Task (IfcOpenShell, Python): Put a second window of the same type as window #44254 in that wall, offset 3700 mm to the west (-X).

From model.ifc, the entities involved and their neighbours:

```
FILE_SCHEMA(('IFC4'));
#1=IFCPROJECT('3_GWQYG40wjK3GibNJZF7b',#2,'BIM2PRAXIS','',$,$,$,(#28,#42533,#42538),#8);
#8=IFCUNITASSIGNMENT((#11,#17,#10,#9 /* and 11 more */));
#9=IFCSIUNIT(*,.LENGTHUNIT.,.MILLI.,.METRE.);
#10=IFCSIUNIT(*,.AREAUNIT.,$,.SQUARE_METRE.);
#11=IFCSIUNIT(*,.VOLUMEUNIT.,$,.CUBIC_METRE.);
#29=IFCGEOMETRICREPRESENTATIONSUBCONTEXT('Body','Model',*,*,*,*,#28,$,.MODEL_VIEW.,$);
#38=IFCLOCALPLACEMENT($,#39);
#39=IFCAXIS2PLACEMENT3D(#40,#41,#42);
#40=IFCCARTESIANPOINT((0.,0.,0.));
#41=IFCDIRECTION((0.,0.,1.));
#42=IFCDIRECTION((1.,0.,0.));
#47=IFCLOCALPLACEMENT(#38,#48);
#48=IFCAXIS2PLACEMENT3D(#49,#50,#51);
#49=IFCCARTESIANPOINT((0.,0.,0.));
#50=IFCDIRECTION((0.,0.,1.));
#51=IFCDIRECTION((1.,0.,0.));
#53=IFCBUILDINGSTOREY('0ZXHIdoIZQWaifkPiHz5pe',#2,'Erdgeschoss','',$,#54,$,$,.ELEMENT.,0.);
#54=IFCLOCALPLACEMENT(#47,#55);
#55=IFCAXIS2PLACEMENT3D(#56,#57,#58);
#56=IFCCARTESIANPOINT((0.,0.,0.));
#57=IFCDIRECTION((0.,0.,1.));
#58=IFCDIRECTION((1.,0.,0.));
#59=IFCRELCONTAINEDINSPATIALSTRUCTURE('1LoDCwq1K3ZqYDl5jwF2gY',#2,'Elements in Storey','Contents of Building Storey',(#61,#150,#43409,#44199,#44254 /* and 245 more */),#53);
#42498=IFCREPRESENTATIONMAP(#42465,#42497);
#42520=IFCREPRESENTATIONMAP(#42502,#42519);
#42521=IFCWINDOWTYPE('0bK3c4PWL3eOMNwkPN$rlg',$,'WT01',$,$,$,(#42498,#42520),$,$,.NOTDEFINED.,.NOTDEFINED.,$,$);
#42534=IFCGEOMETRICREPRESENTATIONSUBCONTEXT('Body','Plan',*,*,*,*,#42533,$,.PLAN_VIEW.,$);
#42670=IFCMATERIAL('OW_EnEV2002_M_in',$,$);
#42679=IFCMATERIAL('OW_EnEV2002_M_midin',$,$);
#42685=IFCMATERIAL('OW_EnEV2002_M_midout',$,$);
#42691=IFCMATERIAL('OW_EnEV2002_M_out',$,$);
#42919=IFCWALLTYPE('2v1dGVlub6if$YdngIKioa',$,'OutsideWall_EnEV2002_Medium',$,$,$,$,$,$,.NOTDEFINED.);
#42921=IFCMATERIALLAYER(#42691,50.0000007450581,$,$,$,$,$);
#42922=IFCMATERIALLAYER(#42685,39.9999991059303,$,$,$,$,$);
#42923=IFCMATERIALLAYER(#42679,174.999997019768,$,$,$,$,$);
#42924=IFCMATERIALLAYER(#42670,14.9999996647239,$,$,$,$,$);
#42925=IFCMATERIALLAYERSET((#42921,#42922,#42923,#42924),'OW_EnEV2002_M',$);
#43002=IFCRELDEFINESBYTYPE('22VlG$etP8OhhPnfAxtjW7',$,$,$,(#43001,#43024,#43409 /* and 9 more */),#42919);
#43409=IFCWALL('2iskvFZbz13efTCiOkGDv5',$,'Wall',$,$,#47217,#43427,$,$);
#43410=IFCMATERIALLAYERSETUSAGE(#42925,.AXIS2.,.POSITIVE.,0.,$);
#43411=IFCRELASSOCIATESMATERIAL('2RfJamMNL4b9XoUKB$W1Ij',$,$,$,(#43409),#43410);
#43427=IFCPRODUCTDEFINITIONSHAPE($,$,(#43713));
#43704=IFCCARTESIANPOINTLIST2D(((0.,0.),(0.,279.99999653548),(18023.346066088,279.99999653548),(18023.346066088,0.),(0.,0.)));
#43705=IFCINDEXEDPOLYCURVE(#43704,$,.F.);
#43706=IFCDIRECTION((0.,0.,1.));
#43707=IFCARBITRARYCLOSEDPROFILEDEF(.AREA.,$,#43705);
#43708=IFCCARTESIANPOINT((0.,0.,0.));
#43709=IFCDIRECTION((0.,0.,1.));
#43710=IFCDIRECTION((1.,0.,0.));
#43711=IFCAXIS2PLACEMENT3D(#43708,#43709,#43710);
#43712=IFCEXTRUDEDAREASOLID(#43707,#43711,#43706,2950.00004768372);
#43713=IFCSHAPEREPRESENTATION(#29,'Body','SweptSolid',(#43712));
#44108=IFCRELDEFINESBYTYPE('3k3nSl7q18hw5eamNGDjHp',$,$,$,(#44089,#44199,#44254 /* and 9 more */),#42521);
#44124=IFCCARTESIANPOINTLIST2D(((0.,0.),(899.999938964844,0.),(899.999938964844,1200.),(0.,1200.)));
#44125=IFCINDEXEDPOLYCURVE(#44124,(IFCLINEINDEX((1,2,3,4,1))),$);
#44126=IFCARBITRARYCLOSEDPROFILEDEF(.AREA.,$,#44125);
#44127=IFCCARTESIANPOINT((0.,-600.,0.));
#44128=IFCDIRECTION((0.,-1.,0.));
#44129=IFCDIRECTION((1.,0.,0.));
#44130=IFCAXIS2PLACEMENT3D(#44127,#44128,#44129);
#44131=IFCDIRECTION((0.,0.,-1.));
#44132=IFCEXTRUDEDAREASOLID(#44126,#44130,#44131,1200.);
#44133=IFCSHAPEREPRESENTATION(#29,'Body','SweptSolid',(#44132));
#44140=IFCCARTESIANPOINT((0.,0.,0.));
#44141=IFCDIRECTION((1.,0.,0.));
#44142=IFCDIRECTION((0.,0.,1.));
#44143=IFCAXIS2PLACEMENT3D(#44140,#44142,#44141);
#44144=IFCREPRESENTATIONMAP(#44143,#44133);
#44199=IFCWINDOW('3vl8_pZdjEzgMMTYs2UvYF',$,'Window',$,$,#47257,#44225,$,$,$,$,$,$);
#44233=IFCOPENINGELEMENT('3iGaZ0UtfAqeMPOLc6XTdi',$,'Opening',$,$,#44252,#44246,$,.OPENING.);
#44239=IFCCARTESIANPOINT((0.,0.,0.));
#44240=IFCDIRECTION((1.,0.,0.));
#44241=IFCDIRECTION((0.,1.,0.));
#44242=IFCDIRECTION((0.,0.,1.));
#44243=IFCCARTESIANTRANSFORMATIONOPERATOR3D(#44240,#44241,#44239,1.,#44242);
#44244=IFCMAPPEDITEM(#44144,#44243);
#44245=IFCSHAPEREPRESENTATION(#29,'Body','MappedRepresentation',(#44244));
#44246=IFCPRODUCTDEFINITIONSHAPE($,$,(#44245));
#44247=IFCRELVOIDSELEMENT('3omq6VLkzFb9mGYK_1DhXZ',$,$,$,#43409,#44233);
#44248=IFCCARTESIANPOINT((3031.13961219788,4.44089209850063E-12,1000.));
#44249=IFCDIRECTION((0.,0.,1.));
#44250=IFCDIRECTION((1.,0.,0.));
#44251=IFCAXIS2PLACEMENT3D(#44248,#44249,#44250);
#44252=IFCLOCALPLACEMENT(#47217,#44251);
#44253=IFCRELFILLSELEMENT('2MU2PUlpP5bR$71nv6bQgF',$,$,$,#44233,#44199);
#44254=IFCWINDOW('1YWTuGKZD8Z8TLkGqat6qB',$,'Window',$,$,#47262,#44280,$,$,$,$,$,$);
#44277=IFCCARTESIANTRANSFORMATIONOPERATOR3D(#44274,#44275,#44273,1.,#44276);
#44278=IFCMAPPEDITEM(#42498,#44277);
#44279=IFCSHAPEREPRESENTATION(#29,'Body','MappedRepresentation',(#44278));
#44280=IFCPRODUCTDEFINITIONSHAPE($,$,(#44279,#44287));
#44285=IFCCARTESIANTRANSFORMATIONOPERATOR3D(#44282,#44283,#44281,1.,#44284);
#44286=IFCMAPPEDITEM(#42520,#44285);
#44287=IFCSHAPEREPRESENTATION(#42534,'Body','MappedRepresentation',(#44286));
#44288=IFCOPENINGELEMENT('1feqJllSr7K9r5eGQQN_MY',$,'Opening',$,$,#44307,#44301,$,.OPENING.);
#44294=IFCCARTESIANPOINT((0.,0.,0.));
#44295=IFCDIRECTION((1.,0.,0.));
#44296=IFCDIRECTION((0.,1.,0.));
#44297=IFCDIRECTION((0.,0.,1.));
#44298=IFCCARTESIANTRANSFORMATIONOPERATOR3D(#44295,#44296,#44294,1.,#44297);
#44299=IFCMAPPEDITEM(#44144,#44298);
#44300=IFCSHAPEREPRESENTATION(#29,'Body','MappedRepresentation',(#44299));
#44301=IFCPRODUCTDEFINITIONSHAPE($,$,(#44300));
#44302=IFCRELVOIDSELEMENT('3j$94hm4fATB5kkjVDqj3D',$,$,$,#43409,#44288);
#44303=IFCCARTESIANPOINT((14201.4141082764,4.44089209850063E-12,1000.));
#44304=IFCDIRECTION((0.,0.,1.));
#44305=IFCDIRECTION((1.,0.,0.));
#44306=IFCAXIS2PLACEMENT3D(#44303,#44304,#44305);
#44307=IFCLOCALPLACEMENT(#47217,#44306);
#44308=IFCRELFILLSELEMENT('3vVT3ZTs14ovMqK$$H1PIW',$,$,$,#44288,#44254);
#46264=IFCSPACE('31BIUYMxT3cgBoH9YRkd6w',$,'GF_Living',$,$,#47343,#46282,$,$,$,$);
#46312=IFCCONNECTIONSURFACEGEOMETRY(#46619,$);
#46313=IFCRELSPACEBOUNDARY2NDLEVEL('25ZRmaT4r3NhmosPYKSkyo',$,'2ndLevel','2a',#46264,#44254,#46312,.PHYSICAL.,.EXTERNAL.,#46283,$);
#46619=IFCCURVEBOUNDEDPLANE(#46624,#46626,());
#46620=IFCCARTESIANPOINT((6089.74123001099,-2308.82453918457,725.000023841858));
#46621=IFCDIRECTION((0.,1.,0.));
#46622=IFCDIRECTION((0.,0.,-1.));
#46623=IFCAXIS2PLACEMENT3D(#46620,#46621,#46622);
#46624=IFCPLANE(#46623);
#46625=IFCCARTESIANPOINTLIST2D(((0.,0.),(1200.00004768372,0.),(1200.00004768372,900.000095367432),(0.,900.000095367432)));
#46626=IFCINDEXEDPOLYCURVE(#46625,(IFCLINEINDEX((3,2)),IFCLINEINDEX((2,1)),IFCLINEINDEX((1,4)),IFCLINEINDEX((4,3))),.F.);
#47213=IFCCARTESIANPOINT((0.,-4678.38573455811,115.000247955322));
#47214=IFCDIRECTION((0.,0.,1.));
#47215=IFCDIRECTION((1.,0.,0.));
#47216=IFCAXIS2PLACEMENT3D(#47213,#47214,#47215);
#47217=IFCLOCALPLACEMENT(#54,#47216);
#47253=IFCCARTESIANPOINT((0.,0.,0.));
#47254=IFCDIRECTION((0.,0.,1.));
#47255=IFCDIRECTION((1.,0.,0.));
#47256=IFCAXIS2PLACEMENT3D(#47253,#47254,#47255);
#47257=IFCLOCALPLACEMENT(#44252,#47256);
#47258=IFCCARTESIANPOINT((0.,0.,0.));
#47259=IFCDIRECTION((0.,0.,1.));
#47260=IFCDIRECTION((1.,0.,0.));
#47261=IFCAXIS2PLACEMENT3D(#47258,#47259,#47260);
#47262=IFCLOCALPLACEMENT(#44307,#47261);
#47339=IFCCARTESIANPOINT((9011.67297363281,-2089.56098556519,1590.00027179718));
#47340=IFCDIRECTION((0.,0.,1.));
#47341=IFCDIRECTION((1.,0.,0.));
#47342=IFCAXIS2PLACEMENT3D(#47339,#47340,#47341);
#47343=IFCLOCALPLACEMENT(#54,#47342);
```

```python
import numpy as np
import ifcopenshell
import ifcopenshell.api.feature
import ifcopenshell.api.geometry
import ifcopenshell.api.root
import ifcopenshell.geom
import ifcopenshell.util.element
import ifcopenshell.util.placement
import ifcopenshell.util.shape
import ifcopenshell.util.unit

model = ifcopenshell.open("model.ifc")
unit_scale = ifcopenshell.util.unit.calculate_unit_scale(model)
settings = ifcopenshell.geom.settings()


def volume(element):
    """Net volume in cubic metres, openings subtracted."""
    shape = ifcopenshell.geom.create_shape(settings, element)
    return ifcopenshell.util.shape.get_volume(shape.geometry)


window = model.by_guid("1YWTuGKZD8Z8TLkGqat6qB")
opening = window.FillsVoids[0].RelatingOpeningElement
wall = opening.VoidsElements[0].RelatingBuildingElement
before = volume(wall)
shift = ifcopenshell.util.placement.get_local_placement(wall.ObjectPlacement)[:3, 0] * -3.7 / unit_scale

# copy_class copies the void relationship, type, container and properties, but no geometry.
new_opening = ifcopenshell.api.root.copy_class(model, product=opening)
new_opening.Representation = ifcopenshell.util.element.copy_deep(
    model, opening.Representation, exclude=["IfcGeometricRepresentationContext", "IfcRepresentationMap"]
)
new_window = ifcopenshell.api.root.copy_class(model, product=window)
new_window.Representation = ifcopenshell.util.element.copy_deep(
    model, window.Representation, exclude=["IfcGeometricRepresentationContext", "IfcRepresentationMap"]
)
ifcopenshell.api.feature.add_filling(model, opening=new_opening, element=new_window)

for old, new in ((opening, new_opening), (window, new_window)):
    matrix = ifcopenshell.util.placement.get_local_placement(old.ObjectPlacement)
    matrix[:3, 3] += shift
    ifcopenshell.api.geometry.edit_object_placement(model, product=new, matrix=matrix, is_si=False)

# The copied space boundaries still share their surfaces with the original.
for rel in new_window.ProvidesBoundaries:
    if rel.ConnectionGeometry:
        rel.ConnectionGeometry = ifcopenshell.util.element.copy_deep(model, rel.ConnectionGeometry)

# Space boundary surfaces are stored in each space's coordinates; move them too.
for rel in new_window.ProvidesBoundaries:
    if not rel.ConnectionGeometry:
        continue
    surface = rel.ConnectionGeometry.SurfaceOnRelatingElement.BasisSurface
    space_matrix = ifcopenshell.util.placement.get_local_placement(rel.RelatingSpace.ObjectPlacement)
    point = np.array(surface.Position.Location.Coordinates) + space_matrix[:3, :3].T @ shift
    surface.Position = model.createIfcAxis2Placement3D(
        model.createIfcCartesianPoint(point.tolist()), surface.Position.Axis, surface.Position.RefDirection
    )

after = volume(wall)

print(f"wall volume {before:.3f} -> {after:.3f} m3")

model.write("model_v2.ifc")
```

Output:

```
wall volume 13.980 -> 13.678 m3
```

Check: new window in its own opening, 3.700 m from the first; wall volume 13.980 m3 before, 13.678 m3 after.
